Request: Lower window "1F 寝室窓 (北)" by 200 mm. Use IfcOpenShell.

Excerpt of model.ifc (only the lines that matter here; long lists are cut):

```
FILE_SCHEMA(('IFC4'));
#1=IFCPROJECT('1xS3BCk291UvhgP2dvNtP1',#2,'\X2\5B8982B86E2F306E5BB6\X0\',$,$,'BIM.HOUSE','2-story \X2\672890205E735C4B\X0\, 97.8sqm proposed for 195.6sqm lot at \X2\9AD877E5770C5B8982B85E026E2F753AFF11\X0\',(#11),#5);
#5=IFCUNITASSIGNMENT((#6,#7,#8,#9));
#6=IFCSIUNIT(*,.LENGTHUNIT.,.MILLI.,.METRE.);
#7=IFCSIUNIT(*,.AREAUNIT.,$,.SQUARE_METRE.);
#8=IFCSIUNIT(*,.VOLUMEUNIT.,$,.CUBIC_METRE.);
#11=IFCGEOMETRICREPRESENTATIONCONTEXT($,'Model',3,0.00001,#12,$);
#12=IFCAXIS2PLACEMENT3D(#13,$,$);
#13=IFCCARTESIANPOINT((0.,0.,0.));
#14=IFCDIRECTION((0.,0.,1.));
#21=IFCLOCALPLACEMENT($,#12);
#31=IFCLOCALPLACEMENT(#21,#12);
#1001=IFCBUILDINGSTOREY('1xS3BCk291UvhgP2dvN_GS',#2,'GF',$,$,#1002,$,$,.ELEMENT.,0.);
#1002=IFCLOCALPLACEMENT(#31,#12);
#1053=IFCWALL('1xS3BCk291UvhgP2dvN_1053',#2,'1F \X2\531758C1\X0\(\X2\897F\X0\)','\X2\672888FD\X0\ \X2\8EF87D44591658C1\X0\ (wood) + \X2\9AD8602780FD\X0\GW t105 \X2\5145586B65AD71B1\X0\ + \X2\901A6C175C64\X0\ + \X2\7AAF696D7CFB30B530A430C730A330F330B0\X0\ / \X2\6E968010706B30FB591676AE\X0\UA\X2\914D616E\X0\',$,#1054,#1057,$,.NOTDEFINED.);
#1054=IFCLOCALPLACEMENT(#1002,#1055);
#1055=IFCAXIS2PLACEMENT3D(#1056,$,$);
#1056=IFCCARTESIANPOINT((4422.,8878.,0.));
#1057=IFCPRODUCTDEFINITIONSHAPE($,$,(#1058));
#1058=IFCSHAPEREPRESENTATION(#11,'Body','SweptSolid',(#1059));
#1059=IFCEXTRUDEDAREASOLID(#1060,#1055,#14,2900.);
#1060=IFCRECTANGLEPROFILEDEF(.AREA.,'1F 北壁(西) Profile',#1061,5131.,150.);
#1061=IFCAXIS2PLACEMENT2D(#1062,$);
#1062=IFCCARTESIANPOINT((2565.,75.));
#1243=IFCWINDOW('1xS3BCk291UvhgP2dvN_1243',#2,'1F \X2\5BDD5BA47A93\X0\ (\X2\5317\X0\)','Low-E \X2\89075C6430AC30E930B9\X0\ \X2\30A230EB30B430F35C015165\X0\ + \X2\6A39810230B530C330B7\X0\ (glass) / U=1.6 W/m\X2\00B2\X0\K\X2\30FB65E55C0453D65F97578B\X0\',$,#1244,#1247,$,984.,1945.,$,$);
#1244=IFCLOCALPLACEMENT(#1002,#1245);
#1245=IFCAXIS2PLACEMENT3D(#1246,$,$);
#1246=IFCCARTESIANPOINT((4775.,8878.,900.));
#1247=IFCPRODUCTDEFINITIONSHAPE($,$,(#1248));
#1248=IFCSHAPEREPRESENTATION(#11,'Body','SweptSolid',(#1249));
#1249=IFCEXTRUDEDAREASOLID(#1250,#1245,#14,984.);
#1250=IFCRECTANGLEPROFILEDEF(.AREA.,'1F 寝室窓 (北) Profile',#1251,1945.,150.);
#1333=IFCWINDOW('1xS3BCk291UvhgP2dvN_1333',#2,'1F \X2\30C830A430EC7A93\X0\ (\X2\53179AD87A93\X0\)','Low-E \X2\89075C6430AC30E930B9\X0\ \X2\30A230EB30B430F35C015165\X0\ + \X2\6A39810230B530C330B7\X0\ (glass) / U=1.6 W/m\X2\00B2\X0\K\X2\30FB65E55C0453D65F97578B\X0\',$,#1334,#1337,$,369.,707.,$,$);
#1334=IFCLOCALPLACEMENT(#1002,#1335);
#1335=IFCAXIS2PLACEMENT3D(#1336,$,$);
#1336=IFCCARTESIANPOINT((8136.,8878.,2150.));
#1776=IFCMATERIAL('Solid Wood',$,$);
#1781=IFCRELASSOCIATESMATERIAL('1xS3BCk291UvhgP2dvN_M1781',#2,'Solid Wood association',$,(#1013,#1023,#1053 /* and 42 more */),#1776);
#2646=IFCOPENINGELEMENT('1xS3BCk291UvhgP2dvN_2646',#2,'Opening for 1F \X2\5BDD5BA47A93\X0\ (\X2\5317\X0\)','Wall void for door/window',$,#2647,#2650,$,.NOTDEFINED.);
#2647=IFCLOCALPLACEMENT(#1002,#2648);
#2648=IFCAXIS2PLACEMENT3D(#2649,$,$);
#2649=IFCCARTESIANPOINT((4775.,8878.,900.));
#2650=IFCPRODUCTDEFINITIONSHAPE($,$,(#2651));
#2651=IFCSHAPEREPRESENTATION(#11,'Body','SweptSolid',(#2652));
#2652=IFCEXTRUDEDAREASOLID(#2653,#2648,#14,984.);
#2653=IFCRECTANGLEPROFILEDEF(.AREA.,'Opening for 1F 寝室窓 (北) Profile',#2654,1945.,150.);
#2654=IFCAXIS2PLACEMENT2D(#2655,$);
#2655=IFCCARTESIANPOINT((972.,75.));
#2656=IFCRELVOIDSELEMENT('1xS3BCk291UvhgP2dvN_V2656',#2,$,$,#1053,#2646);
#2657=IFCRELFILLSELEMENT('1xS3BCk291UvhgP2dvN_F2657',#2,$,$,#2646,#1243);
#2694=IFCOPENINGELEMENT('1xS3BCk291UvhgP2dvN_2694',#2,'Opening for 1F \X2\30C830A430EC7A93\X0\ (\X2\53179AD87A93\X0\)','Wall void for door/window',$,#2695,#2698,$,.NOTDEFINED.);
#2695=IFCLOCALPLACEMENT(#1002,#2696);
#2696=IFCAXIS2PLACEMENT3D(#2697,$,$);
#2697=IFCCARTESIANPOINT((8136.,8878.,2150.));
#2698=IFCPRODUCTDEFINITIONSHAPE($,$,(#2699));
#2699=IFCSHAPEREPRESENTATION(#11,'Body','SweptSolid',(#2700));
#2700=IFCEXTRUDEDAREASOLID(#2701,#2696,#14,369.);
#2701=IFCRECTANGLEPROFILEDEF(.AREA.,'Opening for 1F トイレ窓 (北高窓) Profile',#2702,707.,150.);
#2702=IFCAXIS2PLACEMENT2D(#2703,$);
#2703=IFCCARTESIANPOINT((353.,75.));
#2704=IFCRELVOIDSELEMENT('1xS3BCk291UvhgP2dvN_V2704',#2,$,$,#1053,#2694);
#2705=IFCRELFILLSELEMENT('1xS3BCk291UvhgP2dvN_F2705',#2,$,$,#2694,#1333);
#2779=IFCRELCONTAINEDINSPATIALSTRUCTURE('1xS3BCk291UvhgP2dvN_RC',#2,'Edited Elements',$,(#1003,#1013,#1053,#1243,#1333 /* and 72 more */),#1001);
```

```python
import numpy as np
import ifcopenshell
import ifcopenshell.api.geometry
import ifcopenshell.util.placement
import ifcopenshell.util.unit

model = ifcopenshell.open("model.ifc")
unit_scale = ifcopenshell.util.unit.calculate_unit_scale(model)

window = model.by_guid("1xS3BCk291UvhgP2dvN_1243")
opening = window.FillsVoids[0].RelatingOpeningElement
dz = -0.2 / unit_scale

shift = np.array([0.0, 0.0, dz])
# The window is not placed relative to its opening, so move both.
for product in (opening, window):
    matrix = ifcopenshell.util.placement.get_local_placement(product.ObjectPlacement)
    matrix[:3, 3] += shift
    ifcopenshell.api.geometry.edit_object_placement(model, product=product, matrix=matrix, is_si=False)

print(f"moved by {dz * unit_scale:+.3f} m")

model.write("model_edited.ifc")
```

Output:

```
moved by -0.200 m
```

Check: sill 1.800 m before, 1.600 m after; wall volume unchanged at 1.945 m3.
